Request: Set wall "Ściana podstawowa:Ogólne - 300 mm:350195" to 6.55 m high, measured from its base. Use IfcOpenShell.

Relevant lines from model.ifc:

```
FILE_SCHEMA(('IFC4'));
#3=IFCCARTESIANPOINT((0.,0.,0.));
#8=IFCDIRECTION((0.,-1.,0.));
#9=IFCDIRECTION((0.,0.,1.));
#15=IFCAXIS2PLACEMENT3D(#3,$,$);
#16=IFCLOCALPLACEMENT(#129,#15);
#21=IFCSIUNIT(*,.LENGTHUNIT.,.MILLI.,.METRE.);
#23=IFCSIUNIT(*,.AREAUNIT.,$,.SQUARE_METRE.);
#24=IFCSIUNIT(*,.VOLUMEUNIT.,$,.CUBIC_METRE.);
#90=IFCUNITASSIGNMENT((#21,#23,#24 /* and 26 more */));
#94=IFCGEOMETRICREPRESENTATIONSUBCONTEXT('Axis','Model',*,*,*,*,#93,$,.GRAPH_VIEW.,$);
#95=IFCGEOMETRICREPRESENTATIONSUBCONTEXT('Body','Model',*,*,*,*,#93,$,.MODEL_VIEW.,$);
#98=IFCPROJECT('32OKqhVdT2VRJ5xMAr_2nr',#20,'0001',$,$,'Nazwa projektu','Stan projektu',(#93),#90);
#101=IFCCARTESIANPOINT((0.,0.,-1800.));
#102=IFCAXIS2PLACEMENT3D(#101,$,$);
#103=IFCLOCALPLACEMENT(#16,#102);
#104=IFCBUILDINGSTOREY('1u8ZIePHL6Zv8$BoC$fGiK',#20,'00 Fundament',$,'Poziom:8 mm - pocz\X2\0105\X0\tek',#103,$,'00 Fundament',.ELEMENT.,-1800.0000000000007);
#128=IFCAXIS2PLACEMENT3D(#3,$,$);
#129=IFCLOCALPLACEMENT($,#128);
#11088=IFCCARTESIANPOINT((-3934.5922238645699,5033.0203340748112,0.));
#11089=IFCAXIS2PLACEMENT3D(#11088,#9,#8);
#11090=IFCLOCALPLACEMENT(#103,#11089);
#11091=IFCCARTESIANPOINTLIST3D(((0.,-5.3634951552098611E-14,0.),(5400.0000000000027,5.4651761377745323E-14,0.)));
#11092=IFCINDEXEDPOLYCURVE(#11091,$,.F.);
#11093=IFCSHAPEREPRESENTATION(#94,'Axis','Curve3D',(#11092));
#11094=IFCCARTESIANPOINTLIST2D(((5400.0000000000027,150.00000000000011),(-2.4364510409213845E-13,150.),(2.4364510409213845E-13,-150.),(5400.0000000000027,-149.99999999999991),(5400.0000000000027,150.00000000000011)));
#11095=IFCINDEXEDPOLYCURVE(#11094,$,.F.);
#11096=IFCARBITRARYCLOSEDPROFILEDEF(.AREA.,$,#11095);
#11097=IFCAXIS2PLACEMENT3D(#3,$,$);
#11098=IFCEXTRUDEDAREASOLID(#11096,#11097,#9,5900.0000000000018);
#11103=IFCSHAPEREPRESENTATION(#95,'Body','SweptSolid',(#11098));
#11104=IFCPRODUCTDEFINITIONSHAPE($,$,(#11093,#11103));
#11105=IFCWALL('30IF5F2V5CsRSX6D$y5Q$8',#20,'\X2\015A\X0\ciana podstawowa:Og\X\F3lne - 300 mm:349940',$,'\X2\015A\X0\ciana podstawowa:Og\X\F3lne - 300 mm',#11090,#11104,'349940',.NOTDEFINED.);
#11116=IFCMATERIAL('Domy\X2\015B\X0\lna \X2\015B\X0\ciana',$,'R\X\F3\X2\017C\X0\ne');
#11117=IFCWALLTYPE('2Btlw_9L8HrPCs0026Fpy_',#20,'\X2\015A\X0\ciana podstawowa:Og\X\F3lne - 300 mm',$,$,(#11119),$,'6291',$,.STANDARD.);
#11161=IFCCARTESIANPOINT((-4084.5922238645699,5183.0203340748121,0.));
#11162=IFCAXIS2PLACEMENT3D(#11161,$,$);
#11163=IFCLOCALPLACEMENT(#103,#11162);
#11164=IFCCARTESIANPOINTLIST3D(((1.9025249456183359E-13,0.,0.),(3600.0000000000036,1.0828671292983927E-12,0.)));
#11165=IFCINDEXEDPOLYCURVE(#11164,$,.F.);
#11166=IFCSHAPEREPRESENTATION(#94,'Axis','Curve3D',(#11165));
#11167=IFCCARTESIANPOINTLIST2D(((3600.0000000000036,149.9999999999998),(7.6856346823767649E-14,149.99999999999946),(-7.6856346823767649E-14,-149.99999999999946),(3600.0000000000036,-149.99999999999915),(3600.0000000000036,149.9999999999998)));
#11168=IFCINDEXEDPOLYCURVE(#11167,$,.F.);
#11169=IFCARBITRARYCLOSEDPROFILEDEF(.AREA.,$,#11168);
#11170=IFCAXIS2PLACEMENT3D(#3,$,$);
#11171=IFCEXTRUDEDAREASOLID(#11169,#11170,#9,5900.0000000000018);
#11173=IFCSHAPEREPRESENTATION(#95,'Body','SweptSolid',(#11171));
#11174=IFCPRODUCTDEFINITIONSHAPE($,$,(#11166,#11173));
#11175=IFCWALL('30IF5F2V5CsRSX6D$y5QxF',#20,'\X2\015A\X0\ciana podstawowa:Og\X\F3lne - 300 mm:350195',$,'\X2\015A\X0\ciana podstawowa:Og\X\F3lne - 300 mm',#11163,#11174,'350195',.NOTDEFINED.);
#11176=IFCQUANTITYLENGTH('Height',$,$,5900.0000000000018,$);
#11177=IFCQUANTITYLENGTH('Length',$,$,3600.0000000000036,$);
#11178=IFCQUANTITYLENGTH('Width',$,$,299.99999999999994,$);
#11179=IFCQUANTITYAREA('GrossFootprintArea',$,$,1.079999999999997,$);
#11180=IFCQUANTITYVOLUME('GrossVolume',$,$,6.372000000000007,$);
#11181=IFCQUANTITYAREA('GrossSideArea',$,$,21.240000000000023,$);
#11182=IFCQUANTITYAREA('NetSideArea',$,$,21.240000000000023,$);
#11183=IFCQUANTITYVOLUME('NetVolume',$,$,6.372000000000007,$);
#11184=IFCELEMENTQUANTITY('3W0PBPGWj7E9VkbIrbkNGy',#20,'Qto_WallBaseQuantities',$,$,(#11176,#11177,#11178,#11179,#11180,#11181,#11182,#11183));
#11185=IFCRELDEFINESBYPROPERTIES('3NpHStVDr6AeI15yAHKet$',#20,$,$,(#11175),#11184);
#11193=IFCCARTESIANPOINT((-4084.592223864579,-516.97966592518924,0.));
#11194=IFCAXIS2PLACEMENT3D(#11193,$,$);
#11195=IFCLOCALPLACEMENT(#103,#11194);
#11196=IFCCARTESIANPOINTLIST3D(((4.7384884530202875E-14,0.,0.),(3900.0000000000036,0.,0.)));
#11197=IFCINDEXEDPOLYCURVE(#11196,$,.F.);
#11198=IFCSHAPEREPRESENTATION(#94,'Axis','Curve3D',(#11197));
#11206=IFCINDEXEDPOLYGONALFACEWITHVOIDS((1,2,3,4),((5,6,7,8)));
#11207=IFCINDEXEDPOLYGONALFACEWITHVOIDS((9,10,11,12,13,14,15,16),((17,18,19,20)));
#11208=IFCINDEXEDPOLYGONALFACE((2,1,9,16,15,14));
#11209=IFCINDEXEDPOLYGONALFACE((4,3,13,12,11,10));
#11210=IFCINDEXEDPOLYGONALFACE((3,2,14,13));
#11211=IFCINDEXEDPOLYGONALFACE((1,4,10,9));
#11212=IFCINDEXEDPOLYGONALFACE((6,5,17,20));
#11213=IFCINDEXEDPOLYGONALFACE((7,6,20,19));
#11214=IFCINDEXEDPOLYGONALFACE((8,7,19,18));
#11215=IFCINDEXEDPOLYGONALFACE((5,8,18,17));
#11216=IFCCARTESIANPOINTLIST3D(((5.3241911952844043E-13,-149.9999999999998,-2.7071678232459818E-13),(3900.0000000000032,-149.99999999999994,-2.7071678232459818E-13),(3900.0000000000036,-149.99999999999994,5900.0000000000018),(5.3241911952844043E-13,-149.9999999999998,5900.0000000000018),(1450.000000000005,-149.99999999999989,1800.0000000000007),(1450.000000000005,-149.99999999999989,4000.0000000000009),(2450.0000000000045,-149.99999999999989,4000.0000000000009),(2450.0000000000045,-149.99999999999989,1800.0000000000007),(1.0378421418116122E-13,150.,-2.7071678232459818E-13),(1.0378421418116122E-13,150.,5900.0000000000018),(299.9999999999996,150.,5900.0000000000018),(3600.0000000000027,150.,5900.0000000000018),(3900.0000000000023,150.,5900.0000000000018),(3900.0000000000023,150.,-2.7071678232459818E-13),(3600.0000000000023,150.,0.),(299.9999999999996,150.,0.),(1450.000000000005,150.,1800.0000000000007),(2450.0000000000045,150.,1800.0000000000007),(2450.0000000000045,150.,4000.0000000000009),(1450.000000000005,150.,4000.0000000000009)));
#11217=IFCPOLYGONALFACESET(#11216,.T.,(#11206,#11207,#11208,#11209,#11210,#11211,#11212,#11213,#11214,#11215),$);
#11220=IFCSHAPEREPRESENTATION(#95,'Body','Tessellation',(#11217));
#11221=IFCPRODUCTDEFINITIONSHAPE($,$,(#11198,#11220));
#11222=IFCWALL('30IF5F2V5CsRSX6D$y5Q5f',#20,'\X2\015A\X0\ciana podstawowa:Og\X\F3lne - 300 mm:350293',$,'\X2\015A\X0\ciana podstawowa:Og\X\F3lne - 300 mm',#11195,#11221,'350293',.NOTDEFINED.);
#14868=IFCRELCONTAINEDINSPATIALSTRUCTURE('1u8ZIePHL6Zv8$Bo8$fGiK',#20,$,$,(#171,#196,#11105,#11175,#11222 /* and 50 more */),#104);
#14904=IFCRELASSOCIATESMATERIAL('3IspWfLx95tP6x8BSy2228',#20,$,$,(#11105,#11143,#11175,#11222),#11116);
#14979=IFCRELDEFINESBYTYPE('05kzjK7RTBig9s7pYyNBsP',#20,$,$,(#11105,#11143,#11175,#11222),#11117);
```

```python
import ifcopenshell
import ifcopenshell.api.pset
import ifcopenshell.geom
import ifcopenshell.util.element
import ifcopenshell.util.representation
import ifcopenshell.util.shape
import ifcopenshell.util.unit

model = ifcopenshell.open("model.ifc")
unit_scale = ifcopenshell.util.unit.calculate_unit_scale(model)
area_scale = ifcopenshell.util.unit.calculate_unit_scale(model, "AREAUNIT")
volume_scale = ifcopenshell.util.unit.calculate_unit_scale(model, "VOLUMEUNIT")
settings = ifcopenshell.geom.settings()


def volume(element):
    """Net volume in cubic metres, openings subtracted."""
    shape = ifcopenshell.geom.create_shape(settings, element)
    return ifcopenshell.util.shape.get_volume(shape.geometry)


wall = model.by_id(11175)
before = volume(wall)

body = ifcopenshell.util.representation.get_representation(wall, "Model", "Body")
solid = body.Items[0]
old_height = solid.Depth
solid.Depth = 6.55 / unit_scale
after = volume(wall)
thickness = 0.3  # wall thickness in metres

# Update the stored height, areas and volumes.
qto = model.by_id(ifcopenshell.util.element.get_pset(wall, "Qto_WallBaseQuantities", should_inherit=False)["id"])
ifcopenshell.api.pset.edit_qto(model, qto=qto, properties={
    "Height": solid.Depth,
    "GrossVolume": ifcopenshell.util.element.get_pset(wall, "Qto_WallBaseQuantities", "GrossVolume") * solid.Depth / old_height,
    "GrossSideArea": ifcopenshell.util.element.get_pset(wall, "Qto_WallBaseQuantities", "GrossSideArea") * solid.Depth / old_height,
    "NetSideArea": after / thickness / area_scale,
    "NetVolume": after / volume_scale,
})

print(f"height {old_height:g} -> {solid.Depth:g}, volume {before:.3f} -> {after:.3f} m3")

model.write("model-out.ifc")
```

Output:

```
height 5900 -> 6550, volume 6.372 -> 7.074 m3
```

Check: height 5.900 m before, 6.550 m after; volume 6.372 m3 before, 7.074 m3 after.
